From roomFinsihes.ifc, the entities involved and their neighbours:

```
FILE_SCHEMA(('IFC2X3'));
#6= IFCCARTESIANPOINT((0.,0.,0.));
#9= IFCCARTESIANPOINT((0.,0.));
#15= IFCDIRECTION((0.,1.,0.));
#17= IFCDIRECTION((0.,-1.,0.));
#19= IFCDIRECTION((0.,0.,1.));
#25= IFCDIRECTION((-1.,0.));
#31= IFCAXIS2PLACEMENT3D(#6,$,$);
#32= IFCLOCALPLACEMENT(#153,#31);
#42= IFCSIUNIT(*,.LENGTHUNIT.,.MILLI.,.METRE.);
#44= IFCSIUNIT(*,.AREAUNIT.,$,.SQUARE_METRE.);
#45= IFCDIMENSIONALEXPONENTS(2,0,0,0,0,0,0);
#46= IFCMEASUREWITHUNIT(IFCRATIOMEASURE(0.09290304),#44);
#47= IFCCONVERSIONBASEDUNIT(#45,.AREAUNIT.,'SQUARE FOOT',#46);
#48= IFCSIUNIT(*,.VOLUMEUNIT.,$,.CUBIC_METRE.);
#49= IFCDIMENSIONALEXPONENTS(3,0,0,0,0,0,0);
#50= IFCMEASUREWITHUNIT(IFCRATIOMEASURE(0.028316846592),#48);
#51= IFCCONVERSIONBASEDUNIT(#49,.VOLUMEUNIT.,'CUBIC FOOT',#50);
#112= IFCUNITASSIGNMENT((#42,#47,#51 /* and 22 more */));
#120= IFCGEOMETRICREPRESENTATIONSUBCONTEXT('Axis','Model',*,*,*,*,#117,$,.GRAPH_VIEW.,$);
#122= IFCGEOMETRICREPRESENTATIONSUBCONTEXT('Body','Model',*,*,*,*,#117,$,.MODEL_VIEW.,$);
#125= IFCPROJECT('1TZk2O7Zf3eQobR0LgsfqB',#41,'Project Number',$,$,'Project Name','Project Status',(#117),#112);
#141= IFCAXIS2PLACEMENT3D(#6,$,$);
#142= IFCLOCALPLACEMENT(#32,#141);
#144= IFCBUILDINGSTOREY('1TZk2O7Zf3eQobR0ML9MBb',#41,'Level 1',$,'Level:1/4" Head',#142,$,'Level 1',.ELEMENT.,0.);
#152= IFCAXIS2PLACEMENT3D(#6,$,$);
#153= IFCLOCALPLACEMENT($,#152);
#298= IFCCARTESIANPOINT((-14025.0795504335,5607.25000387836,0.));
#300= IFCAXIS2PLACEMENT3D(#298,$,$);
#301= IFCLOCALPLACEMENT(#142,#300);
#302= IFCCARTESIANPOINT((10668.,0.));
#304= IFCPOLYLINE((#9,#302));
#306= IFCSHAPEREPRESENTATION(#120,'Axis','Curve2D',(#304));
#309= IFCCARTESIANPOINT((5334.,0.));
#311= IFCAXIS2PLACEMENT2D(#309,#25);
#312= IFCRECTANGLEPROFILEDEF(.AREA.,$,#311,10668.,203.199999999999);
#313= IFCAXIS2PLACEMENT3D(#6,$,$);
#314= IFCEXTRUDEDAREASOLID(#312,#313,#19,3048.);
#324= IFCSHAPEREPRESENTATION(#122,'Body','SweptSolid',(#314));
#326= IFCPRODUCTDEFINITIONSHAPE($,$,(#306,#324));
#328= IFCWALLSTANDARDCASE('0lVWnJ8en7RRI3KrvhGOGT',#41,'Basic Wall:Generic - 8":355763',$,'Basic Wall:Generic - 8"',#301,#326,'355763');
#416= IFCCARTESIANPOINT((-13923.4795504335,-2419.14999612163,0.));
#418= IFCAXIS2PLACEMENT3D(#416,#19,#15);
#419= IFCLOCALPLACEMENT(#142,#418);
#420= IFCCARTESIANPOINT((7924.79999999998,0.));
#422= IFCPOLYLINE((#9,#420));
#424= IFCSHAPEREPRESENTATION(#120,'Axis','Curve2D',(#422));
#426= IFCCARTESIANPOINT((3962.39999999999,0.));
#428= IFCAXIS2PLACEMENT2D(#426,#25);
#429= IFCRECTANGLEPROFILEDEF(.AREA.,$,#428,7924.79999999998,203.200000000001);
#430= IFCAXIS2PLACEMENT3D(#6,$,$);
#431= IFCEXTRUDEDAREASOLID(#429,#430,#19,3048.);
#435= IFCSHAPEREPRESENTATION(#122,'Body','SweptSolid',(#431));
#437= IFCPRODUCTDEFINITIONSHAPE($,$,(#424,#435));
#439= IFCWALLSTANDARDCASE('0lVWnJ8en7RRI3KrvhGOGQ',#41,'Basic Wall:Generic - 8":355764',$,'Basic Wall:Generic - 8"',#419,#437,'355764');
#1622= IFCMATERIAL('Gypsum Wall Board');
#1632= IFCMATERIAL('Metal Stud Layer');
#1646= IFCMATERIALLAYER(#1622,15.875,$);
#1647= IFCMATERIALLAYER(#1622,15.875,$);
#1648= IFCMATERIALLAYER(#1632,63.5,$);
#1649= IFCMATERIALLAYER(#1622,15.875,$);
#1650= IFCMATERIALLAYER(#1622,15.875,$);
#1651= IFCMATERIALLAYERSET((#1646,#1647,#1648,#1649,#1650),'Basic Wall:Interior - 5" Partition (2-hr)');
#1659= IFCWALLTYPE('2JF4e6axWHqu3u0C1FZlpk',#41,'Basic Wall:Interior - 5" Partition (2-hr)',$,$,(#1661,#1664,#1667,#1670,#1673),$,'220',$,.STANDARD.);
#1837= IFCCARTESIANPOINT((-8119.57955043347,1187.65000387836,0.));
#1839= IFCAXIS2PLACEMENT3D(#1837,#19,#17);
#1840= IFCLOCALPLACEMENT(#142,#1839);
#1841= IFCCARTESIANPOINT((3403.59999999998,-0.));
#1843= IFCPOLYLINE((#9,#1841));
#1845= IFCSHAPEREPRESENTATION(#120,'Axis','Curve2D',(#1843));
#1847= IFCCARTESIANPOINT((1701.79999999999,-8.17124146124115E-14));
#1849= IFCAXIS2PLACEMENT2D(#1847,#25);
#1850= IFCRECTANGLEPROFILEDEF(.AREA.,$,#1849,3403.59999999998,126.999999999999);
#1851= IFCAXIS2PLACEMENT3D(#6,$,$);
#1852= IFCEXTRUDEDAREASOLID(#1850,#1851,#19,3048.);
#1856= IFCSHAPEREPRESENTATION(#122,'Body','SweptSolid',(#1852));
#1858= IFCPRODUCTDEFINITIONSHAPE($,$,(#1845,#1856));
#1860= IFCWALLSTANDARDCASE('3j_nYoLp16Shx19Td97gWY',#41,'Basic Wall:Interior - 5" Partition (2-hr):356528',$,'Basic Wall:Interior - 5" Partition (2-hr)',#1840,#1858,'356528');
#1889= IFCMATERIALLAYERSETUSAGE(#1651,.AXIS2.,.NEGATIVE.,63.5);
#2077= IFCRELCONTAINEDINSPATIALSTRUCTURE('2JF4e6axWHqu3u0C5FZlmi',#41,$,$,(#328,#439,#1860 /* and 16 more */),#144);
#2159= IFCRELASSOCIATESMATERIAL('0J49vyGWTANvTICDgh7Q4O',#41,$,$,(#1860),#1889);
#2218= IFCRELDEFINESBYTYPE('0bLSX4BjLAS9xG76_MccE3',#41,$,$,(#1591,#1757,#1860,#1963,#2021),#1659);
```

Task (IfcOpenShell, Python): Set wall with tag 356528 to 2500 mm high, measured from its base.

```python
import ifcopenshell
import ifcopenshell.geom
import ifcopenshell.util.representation
import ifcopenshell.util.shape

model = ifcopenshell.open("roomFinsihes.ifc")
settings = ifcopenshell.geom.settings()


def volume(element):
    """Net volume in cubic metres, openings subtracted."""
    shape = ifcopenshell.geom.create_shape(settings, element)
    return ifcopenshell.util.shape.get_volume(shape.geometry)


wall = model.by_guid("3j_nYoLp16Shx19Td97gWY")
before = volume(wall)

body = ifcopenshell.util.representation.get_representation(wall, "Model", "Body")
solid = body.Items[0]
old_height = solid.Depth
solid.Depth = 2500.0
after = volume(wall)

print(f"height {old_height:g} -> {solid.Depth:g}, volume {before:.3f} -> {after:.3f} m3")

model.write("roomFinsihes_v2.ifc")
```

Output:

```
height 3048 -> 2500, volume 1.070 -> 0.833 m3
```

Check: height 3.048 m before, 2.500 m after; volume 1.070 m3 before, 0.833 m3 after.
